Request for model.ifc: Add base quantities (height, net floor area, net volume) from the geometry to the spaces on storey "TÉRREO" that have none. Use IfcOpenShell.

First a look at what the model holds.

```python
import ifcopenshell
import ifcopenshell.util.element
import ifcopenshell.util.unit

model = ifcopenshell.open("model.ifc")
print(model.schema)
for unit_type in ("LENGTHUNIT", "AREAUNIT", "VOLUMEUNIT"):
    print(unit_type, ifcopenshell.util.unit.calculate_unit_scale(model, unit_type))
storey = next(s for s in model.by_type("IfcBuildingStorey") if s.Name == "TÉRREO")
spaces = [e for e in ifcopenshell.util.element.get_decomposition(storey) if e.is_a("IfcSpace")]
for e in sorted(spaces, key=lambda e: e.id()):
    print(e.id(), e.is_a(), e.Name, list(ifcopenshell.util.element.get_psets(e, qtos_only=True)), sep=" | ")
```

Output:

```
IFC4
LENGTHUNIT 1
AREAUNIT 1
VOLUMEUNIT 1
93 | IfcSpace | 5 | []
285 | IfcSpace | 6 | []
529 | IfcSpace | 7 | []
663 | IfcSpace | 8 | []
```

```python
import ifcopenshell
import ifcopenshell.api.pset
import ifcopenshell.geom
import ifcopenshell.util.element
import ifcopenshell.util.shape
import ifcopenshell.util.unit

model = ifcopenshell.open("model.ifc")
unit_scale = ifcopenshell.util.unit.calculate_unit_scale(model)
area_scale = ifcopenshell.util.unit.calculate_unit_scale(model, "AREAUNIT")
volume_scale = ifcopenshell.util.unit.calculate_unit_scale(model, "VOLUMEUNIT")
settings = ifcopenshell.geom.settings()

storey = next(s for s in model.by_type("IfcBuildingStorey") if s.Name == "TÉRREO")
spaces = [e for e in ifcopenshell.util.element.get_decomposition(storey) if e.is_a("IfcSpace")]

for e in sorted(spaces, key=lambda e: e.id()):
    if ifcopenshell.util.element.get_psets(e, qtos_only=True, should_inherit=False):
        continue
    # Geometry comes back in metres, in the element's own axes.
    shape = ifcopenshell.geom.create_shape(settings, e)
    values = {
        "Height": ifcopenshell.util.shape.get_z(shape.geometry) / unit_scale,
        "NetFloorArea": ifcopenshell.util.shape.get_footprint_area(shape.geometry) / area_scale,
        "NetVolume": ifcopenshell.util.shape.get_volume(shape.geometry) / volume_scale,
    }
    qto = ifcopenshell.api.pset.add_qto(model, product=e, name="Qto_SpaceBaseQuantities")
    ifcopenshell.api.pset.edit_qto(model, qto=qto, properties=values)
    print(e.id(), {k: round(v, 3) for k, v in values.items()})

model.write("model_rev.ifc")
```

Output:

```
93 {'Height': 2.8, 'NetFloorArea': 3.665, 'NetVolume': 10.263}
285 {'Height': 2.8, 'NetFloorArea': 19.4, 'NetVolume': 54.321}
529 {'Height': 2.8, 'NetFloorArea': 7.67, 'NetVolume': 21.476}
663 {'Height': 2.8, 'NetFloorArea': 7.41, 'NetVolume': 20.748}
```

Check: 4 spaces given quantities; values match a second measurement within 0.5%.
